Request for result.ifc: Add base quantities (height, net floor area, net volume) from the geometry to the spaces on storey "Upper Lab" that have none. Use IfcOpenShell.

First a look at what the model holds.

```python
import ifcopenshell
import ifcopenshell.util.element
import ifcopenshell.util.unit

model = ifcopenshell.open("result.ifc")
print(model.schema)
for unit_type in ("LENGTHUNIT", "AREAUNIT", "VOLUMEUNIT"):
    print(unit_type, ifcopenshell.util.unit.calculate_unit_scale(model, unit_type))
storey = next(s for s in model.by_type("IfcBuildingStorey") if s.Name == "Upper Lab")
spaces = [e for e in ifcopenshell.util.element.get_decomposition(storey) if e.is_a("IfcSpace")]
for e in sorted(spaces, key=lambda e: e.id()):
    print(e.id(), e.is_a(), e.Name, list(ifcopenshell.util.element.get_psets(e, qtos_only=True)), sep=" | ")
```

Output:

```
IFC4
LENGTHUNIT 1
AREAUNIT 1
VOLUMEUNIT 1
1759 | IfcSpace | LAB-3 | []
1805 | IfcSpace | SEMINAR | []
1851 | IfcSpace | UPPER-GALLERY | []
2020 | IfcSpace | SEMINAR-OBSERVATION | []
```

```python
import ifcopenshell
import ifcopenshell.api.pset
import ifcopenshell.geom
import ifcopenshell.util.element
import ifcopenshell.util.shape
import ifcopenshell.util.unit

model = ifcopenshell.open("result.ifc")
unit_scale = ifcopenshell.util.unit.calculate_unit_scale(model)
area_scale = ifcopenshell.util.unit.calculate_unit_scale(model, "AREAUNIT")
volume_scale = ifcopenshell.util.unit.calculate_unit_scale(model, "VOLUMEUNIT")
settings = ifcopenshell.geom.settings()

storey = next(s for s in model.by_type("IfcBuildingStorey") if s.Name == "Upper Lab")
spaces = [e for e in ifcopenshell.util.element.get_decomposition(storey) if e.is_a("IfcSpace")]

for e in sorted(spaces, key=lambda e: e.id()):
    if ifcopenshell.util.element.get_psets(e, qtos_only=True, should_inherit=False):
        continue
    # Geometry comes back in metres, in the element's own axes.
    shape = ifcopenshell.geom.create_shape(settings, e)
    values = {
        "Height": ifcopenshell.util.shape.get_z(shape.geometry) / unit_scale,
        "NetFloorArea": ifcopenshell.util.shape.get_footprint_area(shape.geometry) / area_scale,
        "NetVolume": ifcopenshell.util.shape.get_volume(shape.geometry) / volume_scale,
    }
    qto = ifcopenshell.api.pset.add_qto(model, product=e, name="Qto_SpaceBaseQuantities")
    ifcopenshell.api.pset.edit_qto(model, qto=qto, properties=values)
    print(e.id(), {k: round(v, 3) for k, v in values.items()})

model.write("result_rev.ifc")
```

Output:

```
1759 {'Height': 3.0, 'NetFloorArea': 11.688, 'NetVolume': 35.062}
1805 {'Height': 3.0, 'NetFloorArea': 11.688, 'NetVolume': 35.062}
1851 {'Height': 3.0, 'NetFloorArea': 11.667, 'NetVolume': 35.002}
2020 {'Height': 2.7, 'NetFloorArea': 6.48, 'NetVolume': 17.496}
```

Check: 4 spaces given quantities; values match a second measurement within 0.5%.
